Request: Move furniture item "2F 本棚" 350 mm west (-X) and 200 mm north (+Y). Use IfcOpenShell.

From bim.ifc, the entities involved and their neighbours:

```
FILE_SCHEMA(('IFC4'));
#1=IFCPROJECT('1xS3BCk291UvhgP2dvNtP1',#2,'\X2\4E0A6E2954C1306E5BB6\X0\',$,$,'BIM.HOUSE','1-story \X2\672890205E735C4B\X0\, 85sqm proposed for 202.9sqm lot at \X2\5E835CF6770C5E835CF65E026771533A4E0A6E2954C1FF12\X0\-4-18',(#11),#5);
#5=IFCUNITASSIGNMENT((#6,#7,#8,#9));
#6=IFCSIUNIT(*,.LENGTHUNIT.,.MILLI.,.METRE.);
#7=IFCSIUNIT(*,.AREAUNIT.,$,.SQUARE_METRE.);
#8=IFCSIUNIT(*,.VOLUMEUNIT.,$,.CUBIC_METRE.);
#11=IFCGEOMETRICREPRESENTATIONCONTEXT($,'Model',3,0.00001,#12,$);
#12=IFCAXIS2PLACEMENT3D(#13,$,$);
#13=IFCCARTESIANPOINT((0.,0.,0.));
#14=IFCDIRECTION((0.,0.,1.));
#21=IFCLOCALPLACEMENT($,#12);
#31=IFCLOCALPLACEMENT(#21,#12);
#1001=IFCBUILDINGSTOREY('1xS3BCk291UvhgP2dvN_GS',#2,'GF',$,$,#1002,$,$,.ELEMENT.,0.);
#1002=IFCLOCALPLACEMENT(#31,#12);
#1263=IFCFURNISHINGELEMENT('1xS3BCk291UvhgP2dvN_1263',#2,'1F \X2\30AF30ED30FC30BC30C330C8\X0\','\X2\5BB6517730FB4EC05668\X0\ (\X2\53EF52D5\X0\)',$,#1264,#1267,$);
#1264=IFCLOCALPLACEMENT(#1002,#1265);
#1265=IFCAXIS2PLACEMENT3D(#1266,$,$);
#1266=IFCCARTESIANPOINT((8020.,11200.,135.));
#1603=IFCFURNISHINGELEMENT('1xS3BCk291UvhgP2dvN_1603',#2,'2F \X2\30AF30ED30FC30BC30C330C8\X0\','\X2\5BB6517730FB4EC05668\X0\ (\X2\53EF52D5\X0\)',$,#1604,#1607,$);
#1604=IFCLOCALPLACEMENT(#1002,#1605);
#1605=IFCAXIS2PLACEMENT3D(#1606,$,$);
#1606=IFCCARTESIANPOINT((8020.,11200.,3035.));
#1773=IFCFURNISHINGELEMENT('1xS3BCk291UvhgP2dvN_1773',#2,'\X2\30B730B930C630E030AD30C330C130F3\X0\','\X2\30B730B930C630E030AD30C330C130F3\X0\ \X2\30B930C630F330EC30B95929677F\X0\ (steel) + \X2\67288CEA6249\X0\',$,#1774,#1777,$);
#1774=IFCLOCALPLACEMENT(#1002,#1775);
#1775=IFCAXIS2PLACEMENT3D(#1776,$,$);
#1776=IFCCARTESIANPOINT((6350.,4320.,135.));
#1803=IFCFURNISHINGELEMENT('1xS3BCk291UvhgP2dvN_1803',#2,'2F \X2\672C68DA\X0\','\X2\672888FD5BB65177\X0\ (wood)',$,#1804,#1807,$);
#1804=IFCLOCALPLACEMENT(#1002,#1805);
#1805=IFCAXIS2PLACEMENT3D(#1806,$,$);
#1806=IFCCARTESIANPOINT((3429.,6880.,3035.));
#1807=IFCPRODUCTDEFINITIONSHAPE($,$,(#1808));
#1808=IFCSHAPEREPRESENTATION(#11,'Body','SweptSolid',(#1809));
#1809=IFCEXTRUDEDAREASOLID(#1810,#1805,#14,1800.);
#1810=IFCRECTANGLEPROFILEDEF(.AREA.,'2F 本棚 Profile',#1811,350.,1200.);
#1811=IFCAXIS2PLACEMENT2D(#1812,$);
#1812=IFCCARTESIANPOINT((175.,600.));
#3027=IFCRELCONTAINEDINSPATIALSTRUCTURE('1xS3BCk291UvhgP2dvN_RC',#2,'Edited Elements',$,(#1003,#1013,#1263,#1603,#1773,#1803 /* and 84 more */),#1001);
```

```python
import ifcopenshell
import ifcopenshell.api.geometry
import ifcopenshell.util.placement
import ifcopenshell.util.unit

model = ifcopenshell.open("bim.ifc")
unit_scale = ifcopenshell.util.unit.calculate_unit_scale(model)

item = model.by_guid("1xS3BCk291UvhgP2dvN_1803")
matrix = ifcopenshell.util.placement.get_local_placement(item.ObjectPlacement)
matrix[0, 3] -= 0.35 / unit_scale
matrix[1, 3] += 0.2 / unit_scale
ifcopenshell.api.geometry.edit_object_placement(model, product=item, matrix=matrix, is_si=False)

print(ifcopenshell.util.placement.get_local_placement(item.ObjectPlacement).round(3) + 0.0)

model.write("bim_updated.ifc")
```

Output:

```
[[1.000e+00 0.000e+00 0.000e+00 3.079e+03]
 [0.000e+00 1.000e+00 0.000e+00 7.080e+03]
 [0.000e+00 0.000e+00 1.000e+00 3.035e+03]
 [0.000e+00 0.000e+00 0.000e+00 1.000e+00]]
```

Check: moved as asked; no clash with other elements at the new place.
